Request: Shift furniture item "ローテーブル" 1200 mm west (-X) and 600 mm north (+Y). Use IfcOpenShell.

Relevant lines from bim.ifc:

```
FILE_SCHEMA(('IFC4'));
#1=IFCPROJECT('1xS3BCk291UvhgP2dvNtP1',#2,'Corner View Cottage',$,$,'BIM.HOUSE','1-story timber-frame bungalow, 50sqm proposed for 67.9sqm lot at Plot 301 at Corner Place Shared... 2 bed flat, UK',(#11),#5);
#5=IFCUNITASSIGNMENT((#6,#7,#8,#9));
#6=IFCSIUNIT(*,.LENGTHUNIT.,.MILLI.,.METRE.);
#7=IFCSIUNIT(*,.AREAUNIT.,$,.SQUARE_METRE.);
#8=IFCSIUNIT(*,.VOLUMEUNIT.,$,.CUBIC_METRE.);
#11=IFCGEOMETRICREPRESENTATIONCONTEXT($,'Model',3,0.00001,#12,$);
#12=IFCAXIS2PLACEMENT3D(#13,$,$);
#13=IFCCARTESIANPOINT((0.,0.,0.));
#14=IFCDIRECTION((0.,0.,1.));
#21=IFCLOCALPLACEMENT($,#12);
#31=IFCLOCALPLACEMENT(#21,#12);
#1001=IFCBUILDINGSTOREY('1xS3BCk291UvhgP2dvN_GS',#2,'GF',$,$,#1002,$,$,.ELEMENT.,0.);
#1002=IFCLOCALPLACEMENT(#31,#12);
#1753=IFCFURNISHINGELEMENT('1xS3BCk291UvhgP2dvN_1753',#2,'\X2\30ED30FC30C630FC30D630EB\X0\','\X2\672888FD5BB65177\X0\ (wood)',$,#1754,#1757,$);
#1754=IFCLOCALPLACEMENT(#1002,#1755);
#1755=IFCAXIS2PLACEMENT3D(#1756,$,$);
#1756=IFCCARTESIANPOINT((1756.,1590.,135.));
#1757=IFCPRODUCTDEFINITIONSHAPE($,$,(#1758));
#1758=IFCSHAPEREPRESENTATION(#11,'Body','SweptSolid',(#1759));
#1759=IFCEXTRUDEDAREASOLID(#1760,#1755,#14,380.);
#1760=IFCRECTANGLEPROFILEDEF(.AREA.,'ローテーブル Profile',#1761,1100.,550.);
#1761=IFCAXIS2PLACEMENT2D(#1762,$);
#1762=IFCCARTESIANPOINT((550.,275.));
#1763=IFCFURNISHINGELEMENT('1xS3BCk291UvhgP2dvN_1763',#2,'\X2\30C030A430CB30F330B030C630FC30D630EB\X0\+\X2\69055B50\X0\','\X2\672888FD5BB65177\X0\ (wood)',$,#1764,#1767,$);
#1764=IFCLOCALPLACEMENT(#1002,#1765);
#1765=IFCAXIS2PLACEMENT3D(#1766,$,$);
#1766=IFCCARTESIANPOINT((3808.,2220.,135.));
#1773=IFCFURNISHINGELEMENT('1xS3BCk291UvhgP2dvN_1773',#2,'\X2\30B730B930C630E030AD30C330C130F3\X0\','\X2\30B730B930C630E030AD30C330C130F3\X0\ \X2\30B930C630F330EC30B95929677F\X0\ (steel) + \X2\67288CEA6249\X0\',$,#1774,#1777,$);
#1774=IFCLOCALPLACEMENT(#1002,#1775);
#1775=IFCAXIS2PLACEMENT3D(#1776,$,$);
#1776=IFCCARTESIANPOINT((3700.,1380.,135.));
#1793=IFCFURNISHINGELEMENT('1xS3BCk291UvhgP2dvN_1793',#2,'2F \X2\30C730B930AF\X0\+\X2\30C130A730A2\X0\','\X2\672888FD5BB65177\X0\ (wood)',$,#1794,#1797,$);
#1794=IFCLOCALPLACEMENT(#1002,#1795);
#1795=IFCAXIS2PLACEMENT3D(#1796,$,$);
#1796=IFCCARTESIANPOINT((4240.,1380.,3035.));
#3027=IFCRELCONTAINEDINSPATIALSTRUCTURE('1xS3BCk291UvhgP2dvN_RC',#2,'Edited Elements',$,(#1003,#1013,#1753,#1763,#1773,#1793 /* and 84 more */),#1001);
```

```python
import ifcopenshell
import ifcopenshell.api.geometry
import ifcopenshell.util.placement

model = ifcopenshell.open("bim.ifc")

item = model.by_guid("1xS3BCk291UvhgP2dvN_1753")
matrix = ifcopenshell.util.placement.get_local_placement(item.ObjectPlacement)
matrix[0, 3] -= 1200.0
matrix[1, 3] += 600.0
ifcopenshell.api.geometry.edit_object_placement(model, product=item, matrix=matrix, is_si=False)

print(ifcopenshell.util.placement.get_local_placement(item.ObjectPlacement).round(3) + 0.0)

model.write("bim_v2.ifc")
```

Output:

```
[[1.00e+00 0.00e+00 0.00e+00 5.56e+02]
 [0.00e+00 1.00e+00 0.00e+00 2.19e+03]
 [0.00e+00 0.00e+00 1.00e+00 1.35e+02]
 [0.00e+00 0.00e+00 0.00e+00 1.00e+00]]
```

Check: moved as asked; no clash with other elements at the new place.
